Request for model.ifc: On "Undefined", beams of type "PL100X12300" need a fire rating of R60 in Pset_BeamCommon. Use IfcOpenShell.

First a look at what the model holds.

```python
import ifcopenshell
import ifcopenshell.util.element

model = ifcopenshell.open("model.ifc")
print(model.schema)
storey = next(s for s in model.by_type("IfcBuildingStorey") if s.Name == "Undefined")
beams = [e for e in ifcopenshell.util.element.get_decomposition(storey) if e.is_a("IfcBeam")]
seen = {}
for e in beams:
    element_type = ifcopenshell.util.element.get_type(e)
    key = (element_type.Name if element_type != e and element_type else None, ifcopenshell.util.element.get_pset(e, "Pset_BeamCommon", "FireRating"))
    seen[key] = seen.get(key, 0) + 1
for (name, value), count in sorted(seen.items(), key=str):
    print(count, "x", name, "|", value)
```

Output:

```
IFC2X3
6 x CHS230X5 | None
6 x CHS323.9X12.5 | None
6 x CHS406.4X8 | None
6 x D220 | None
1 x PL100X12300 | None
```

```python
import ifcopenshell
import ifcopenshell.api.pset
import ifcopenshell.util.element

model = ifcopenshell.open("model.ifc")

storey = next(s for s in model.by_type("IfcBuildingStorey") if s.Name == "Undefined")
beams = [e for e in ifcopenshell.util.element.get_decomposition(storey) if e.is_a("IfcBeam")]

count = 0
for e in beams:
    element_type = ifcopenshell.util.element.get_type(e)
    if element_type in (None, e) or element_type.Name != "PL100X12300":
        continue
    # add_pset returns the element's existing set when there is one.
    pset = ifcopenshell.api.pset.add_pset(model, product=e, name="Pset_BeamCommon")
    ifcopenshell.api.pset.edit_pset(model, pset=pset, properties={"FireRating": "R60"})
    count += 1

print(count, "beams updated")

model.write("model_edited.ifc")
```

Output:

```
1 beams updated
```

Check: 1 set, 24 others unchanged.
